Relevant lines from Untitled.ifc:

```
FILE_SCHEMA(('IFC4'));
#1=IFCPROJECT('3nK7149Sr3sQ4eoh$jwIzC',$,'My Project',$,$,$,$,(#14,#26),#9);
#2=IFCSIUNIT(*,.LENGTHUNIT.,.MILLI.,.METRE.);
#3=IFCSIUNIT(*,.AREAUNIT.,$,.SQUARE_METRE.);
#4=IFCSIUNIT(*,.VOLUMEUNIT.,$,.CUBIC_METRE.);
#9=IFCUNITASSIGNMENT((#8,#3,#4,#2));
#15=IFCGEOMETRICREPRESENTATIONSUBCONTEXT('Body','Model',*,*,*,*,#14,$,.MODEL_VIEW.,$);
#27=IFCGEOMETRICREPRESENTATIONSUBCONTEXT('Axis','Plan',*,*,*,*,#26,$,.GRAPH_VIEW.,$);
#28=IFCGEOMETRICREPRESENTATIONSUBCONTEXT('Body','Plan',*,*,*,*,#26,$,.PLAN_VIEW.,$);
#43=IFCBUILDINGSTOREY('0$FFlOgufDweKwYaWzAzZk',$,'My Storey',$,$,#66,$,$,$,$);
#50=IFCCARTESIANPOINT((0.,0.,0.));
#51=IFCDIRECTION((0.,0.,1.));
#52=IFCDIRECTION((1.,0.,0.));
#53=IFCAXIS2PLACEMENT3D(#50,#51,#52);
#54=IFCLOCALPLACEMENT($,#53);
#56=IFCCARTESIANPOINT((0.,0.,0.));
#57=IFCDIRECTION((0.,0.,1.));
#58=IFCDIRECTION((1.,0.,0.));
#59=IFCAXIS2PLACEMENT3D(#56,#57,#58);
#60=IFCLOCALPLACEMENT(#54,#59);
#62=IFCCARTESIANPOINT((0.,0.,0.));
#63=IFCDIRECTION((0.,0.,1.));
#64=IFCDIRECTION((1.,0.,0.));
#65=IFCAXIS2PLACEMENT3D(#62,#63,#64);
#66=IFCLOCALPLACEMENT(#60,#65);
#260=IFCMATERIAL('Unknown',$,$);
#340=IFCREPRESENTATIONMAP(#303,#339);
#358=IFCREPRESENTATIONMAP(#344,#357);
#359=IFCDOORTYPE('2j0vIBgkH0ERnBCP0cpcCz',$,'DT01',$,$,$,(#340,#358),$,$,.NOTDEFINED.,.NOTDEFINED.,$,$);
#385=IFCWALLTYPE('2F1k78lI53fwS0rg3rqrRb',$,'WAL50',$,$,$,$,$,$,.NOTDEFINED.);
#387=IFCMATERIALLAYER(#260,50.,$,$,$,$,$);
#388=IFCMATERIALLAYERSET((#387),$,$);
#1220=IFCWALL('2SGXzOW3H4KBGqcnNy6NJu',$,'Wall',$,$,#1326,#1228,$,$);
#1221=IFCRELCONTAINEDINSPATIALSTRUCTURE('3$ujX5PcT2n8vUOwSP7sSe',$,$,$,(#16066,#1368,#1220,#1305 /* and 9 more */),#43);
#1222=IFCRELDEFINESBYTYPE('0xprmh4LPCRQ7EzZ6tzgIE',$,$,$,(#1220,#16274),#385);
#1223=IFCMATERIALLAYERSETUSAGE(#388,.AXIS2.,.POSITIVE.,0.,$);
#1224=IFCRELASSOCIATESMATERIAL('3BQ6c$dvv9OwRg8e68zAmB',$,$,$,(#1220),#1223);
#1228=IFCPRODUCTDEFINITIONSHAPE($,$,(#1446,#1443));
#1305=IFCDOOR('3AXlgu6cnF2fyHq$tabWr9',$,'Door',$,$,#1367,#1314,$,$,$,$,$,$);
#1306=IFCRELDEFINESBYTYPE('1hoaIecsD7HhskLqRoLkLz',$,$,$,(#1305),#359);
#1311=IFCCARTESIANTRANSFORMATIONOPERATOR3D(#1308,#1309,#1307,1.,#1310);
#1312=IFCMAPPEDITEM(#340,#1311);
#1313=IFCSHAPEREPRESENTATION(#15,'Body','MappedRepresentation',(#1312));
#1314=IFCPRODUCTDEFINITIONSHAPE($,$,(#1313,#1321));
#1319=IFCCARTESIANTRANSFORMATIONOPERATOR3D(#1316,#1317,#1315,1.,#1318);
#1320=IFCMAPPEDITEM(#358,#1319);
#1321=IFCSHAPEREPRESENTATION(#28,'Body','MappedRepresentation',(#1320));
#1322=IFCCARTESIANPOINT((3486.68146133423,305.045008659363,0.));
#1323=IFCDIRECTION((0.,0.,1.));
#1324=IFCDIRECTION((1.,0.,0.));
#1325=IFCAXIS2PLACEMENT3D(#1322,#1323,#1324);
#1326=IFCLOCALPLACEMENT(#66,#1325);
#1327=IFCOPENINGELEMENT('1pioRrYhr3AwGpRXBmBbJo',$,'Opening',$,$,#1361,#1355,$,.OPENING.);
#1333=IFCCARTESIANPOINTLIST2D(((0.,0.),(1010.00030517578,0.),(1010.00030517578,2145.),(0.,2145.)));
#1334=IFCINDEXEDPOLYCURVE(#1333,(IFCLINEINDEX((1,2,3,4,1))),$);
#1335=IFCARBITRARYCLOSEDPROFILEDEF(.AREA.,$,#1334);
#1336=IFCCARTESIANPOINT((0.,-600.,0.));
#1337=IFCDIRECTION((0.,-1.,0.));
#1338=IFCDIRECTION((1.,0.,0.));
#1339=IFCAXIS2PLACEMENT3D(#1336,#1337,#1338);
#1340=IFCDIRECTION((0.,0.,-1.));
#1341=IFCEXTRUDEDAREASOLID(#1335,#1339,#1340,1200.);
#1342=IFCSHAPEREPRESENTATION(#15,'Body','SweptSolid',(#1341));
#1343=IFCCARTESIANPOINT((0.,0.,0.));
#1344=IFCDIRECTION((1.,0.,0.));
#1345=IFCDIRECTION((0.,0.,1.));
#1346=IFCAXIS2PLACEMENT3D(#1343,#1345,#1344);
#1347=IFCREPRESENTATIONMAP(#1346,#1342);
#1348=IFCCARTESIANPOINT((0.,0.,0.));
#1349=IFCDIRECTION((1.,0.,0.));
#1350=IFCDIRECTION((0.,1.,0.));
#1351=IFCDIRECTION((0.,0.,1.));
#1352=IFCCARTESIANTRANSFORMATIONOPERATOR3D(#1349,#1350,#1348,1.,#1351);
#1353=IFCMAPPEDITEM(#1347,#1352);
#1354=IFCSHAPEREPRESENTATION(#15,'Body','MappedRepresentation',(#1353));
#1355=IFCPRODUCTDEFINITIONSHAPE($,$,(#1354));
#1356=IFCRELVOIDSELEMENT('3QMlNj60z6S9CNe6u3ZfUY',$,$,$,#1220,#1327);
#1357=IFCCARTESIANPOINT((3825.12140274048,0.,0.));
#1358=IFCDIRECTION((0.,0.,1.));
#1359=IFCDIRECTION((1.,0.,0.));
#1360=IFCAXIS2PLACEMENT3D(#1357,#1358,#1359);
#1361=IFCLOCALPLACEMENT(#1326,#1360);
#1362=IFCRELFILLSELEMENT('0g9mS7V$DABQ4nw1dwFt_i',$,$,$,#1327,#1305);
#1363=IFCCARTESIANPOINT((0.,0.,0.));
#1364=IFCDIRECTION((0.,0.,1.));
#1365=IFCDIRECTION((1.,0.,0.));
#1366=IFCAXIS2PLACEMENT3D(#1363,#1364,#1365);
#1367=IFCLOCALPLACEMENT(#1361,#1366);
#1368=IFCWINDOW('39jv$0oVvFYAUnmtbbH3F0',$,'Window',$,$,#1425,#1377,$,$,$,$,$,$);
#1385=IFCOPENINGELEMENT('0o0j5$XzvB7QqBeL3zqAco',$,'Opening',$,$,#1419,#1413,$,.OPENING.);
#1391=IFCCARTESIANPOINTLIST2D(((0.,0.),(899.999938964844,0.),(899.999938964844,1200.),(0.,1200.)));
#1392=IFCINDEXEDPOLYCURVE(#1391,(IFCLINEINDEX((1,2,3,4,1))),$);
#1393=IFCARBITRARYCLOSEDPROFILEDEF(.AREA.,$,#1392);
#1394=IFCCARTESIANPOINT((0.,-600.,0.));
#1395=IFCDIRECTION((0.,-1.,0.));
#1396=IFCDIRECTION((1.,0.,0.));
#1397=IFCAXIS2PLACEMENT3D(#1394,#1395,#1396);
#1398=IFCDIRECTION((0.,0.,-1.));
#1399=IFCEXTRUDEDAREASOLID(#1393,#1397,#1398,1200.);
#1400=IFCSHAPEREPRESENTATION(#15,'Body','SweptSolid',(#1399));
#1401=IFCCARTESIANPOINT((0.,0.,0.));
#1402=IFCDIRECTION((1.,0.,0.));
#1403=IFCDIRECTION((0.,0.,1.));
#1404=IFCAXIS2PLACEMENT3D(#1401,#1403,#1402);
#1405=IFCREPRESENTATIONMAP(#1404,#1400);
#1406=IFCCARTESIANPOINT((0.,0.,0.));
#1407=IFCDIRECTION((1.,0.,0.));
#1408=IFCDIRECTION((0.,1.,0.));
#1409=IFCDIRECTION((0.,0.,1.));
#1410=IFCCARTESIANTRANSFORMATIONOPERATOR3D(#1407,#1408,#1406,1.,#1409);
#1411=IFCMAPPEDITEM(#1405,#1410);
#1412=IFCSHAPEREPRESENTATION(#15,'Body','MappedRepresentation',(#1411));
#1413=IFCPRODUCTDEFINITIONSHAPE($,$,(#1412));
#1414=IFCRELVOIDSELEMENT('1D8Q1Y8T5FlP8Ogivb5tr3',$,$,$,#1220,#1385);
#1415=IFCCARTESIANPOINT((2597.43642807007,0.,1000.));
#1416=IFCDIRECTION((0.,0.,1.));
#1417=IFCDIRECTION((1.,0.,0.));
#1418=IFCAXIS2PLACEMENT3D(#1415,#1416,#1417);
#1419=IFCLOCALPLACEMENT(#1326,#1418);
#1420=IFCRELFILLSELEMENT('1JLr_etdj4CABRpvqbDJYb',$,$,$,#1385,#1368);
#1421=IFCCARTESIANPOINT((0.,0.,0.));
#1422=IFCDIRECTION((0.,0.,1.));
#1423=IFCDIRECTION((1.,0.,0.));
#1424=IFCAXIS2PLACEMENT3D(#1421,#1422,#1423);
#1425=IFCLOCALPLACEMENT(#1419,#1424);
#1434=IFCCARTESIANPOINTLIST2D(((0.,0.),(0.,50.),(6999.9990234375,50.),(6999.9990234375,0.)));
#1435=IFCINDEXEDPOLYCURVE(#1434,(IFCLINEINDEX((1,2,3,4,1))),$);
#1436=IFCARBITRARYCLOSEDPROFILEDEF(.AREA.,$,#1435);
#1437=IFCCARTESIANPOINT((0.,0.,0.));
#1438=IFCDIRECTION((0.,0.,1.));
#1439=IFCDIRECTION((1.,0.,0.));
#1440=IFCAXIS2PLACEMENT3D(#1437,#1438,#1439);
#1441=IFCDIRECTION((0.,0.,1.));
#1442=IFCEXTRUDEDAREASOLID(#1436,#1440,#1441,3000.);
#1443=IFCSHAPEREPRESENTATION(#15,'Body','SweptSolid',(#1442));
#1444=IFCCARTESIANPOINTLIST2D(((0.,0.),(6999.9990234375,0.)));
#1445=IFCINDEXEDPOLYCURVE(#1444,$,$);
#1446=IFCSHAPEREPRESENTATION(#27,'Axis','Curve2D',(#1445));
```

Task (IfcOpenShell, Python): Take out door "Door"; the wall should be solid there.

```python
import ifcopenshell
import ifcopenshell.api.feature
import ifcopenshell.api.root
import ifcopenshell.geom
import ifcopenshell.util.shape

model = ifcopenshell.open("Untitled.ifc")
settings = ifcopenshell.geom.settings()


def volume(element):
    """Net volume in cubic metres, openings subtracted."""
    shape = ifcopenshell.geom.create_shape(settings, element)
    return ifcopenshell.util.shape.get_volume(shape.geometry)


door = model.by_id(1305)
opening = door.FillsVoids[0].RelatingOpeningElement
wall = opening.VoidsElements[0].RelatingBuildingElement
before = volume(wall)

ifcopenshell.api.root.remove_product(model, product=door)
ifcopenshell.api.feature.remove_feature(model, feature=opening)

after = volume(wall)

print(f"wall volume {before:.3f} -> {after:.3f} m3")

model.write("Untitled_v2.ifc")
```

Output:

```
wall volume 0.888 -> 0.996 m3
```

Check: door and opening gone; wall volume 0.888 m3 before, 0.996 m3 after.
